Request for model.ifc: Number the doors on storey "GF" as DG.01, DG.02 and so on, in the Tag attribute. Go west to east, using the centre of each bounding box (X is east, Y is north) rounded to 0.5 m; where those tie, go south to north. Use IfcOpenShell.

First a look at what the model holds.

```python
import ifcopenshell
import ifcopenshell.util.element
import ifcopenshell.util.placement

model = ifcopenshell.open("model.ifc")
print(model.schema)
storey = next(s for s in model.by_type("IfcBuildingStorey") if s.Name == "GF")
doors = [e for e in ifcopenshell.util.element.get_decomposition(storey) if e.is_a("IfcDoor")]
for e in sorted(doors, key=lambda e: e.id()):
    origin = ifcopenshell.util.placement.get_local_placement(e.ObjectPlacement)[:3, 3]
    print(e.id(), e.Tag, e.Name, origin.round(2) + 0.0, sep=" | ")
```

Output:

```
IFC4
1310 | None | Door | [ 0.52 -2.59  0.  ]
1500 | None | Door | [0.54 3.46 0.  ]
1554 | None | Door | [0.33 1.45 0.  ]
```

```python
import ifcopenshell
import ifcopenshell.geom
import ifcopenshell.util.element
import ifcopenshell.util.shape

model = ifcopenshell.open("model.ifc")
settings = ifcopenshell.geom.settings()
settings.set("use-world-coords", True)


def centre(element):
    shape = ifcopenshell.geom.create_shape(settings, element)
    return ifcopenshell.util.shape.get_bbox_centroid(shape.geometry)


storey = next(s for s in model.by_type("IfcBuildingStorey") if s.Name == "GF")
doors = [e for e in ifcopenshell.util.element.get_decomposition(storey) if e.is_a("IfcDoor")]

# Insertion points can sit at a corner or the storey origin, so sort by the geometry (in metres).
centres = {e: centre(e) for e in doors}
doors.sort(key=lambda e: (round(centres[e][0] / 0.5), centres[e][1]))

for i, e in enumerate(doors, start=1):
    number = f"DG.{i:02d}"
    e.Tag = number
    print(e.id(), number)

model.write("model_updated.ifc")
```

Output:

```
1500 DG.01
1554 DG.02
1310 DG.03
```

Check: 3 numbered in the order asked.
